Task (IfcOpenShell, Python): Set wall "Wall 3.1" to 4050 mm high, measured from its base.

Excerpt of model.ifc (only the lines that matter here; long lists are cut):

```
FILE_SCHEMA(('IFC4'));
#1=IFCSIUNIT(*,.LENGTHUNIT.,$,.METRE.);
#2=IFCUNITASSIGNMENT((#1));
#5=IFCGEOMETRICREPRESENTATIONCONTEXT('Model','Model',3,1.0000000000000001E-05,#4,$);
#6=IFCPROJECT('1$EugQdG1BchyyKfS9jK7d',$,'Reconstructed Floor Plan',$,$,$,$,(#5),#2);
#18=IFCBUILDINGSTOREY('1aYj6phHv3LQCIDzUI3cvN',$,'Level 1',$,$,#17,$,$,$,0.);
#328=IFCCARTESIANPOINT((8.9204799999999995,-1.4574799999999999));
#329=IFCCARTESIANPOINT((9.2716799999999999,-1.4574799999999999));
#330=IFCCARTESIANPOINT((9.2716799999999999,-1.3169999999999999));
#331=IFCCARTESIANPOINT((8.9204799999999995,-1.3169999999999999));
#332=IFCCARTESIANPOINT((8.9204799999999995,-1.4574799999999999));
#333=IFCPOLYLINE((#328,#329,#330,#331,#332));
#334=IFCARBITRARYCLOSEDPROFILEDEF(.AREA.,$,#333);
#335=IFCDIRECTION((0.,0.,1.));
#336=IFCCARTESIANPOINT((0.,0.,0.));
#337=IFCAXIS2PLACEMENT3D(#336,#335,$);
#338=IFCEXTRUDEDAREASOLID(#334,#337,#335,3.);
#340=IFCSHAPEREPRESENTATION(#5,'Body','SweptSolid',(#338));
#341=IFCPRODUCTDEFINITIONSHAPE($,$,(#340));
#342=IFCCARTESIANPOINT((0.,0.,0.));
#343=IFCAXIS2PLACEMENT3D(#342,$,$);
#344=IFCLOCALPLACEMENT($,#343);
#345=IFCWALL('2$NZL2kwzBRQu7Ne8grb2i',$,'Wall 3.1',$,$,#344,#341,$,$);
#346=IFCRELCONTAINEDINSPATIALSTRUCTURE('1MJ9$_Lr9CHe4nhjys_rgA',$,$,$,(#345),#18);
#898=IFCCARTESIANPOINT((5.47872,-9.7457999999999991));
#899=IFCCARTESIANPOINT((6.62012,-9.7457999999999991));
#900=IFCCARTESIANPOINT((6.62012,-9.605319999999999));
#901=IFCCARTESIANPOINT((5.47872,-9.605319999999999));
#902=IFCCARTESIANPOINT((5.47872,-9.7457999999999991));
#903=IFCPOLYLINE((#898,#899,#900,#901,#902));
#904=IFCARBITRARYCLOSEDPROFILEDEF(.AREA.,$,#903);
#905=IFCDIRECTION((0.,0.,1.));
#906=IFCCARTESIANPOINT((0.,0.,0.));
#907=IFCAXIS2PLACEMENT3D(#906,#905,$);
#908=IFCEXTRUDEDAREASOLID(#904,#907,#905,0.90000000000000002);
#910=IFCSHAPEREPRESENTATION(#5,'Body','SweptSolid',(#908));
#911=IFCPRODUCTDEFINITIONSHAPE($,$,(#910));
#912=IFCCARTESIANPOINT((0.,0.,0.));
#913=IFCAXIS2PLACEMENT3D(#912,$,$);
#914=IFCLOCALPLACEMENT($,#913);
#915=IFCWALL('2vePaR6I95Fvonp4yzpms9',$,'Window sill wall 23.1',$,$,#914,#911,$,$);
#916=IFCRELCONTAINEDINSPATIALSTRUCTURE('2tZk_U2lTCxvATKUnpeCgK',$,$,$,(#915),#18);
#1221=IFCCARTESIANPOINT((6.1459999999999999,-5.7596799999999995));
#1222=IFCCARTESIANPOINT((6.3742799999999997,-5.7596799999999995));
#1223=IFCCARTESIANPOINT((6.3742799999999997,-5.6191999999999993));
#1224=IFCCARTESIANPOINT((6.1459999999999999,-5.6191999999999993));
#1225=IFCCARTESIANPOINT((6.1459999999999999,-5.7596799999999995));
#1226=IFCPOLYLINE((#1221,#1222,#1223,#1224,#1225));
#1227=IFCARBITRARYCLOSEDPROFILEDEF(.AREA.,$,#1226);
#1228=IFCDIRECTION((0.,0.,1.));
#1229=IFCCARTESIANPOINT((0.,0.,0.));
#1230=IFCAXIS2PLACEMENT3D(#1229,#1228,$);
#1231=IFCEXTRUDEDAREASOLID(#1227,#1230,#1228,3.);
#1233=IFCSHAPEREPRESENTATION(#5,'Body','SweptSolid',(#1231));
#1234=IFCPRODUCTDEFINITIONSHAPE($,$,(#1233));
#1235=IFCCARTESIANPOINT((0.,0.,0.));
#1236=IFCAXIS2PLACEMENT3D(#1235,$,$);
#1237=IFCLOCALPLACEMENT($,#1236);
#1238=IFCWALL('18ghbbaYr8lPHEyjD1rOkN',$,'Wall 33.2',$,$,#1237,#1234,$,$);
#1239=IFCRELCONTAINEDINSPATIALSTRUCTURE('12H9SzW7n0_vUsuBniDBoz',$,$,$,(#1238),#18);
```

```python
import ifcopenshell
import ifcopenshell.geom
import ifcopenshell.util.shape

model = ifcopenshell.open("model.ifc")
settings = ifcopenshell.geom.settings()


def volume(element):
    """Net volume in cubic metres, openings subtracted."""
    shape = ifcopenshell.geom.create_shape(settings, element)
    return ifcopenshell.util.shape.get_volume(shape.geometry)


wall = model.by_guid("2$NZL2kwzBRQu7Ne8grb2i")
before = volume(wall)

body = next(r for r in wall.Representation.Representations if r.RepresentationIdentifier == "Body")
solid = body.Items[0]
old_height = solid.Depth
solid.Depth = 4.05
after = volume(wall)

print(f"height {old_height:g} -> {solid.Depth:g}, volume {before:.3f} -> {after:.3f} m3")

model.write("model_v2.ifc")
```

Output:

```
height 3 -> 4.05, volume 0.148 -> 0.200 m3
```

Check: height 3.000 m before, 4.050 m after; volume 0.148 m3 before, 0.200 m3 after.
